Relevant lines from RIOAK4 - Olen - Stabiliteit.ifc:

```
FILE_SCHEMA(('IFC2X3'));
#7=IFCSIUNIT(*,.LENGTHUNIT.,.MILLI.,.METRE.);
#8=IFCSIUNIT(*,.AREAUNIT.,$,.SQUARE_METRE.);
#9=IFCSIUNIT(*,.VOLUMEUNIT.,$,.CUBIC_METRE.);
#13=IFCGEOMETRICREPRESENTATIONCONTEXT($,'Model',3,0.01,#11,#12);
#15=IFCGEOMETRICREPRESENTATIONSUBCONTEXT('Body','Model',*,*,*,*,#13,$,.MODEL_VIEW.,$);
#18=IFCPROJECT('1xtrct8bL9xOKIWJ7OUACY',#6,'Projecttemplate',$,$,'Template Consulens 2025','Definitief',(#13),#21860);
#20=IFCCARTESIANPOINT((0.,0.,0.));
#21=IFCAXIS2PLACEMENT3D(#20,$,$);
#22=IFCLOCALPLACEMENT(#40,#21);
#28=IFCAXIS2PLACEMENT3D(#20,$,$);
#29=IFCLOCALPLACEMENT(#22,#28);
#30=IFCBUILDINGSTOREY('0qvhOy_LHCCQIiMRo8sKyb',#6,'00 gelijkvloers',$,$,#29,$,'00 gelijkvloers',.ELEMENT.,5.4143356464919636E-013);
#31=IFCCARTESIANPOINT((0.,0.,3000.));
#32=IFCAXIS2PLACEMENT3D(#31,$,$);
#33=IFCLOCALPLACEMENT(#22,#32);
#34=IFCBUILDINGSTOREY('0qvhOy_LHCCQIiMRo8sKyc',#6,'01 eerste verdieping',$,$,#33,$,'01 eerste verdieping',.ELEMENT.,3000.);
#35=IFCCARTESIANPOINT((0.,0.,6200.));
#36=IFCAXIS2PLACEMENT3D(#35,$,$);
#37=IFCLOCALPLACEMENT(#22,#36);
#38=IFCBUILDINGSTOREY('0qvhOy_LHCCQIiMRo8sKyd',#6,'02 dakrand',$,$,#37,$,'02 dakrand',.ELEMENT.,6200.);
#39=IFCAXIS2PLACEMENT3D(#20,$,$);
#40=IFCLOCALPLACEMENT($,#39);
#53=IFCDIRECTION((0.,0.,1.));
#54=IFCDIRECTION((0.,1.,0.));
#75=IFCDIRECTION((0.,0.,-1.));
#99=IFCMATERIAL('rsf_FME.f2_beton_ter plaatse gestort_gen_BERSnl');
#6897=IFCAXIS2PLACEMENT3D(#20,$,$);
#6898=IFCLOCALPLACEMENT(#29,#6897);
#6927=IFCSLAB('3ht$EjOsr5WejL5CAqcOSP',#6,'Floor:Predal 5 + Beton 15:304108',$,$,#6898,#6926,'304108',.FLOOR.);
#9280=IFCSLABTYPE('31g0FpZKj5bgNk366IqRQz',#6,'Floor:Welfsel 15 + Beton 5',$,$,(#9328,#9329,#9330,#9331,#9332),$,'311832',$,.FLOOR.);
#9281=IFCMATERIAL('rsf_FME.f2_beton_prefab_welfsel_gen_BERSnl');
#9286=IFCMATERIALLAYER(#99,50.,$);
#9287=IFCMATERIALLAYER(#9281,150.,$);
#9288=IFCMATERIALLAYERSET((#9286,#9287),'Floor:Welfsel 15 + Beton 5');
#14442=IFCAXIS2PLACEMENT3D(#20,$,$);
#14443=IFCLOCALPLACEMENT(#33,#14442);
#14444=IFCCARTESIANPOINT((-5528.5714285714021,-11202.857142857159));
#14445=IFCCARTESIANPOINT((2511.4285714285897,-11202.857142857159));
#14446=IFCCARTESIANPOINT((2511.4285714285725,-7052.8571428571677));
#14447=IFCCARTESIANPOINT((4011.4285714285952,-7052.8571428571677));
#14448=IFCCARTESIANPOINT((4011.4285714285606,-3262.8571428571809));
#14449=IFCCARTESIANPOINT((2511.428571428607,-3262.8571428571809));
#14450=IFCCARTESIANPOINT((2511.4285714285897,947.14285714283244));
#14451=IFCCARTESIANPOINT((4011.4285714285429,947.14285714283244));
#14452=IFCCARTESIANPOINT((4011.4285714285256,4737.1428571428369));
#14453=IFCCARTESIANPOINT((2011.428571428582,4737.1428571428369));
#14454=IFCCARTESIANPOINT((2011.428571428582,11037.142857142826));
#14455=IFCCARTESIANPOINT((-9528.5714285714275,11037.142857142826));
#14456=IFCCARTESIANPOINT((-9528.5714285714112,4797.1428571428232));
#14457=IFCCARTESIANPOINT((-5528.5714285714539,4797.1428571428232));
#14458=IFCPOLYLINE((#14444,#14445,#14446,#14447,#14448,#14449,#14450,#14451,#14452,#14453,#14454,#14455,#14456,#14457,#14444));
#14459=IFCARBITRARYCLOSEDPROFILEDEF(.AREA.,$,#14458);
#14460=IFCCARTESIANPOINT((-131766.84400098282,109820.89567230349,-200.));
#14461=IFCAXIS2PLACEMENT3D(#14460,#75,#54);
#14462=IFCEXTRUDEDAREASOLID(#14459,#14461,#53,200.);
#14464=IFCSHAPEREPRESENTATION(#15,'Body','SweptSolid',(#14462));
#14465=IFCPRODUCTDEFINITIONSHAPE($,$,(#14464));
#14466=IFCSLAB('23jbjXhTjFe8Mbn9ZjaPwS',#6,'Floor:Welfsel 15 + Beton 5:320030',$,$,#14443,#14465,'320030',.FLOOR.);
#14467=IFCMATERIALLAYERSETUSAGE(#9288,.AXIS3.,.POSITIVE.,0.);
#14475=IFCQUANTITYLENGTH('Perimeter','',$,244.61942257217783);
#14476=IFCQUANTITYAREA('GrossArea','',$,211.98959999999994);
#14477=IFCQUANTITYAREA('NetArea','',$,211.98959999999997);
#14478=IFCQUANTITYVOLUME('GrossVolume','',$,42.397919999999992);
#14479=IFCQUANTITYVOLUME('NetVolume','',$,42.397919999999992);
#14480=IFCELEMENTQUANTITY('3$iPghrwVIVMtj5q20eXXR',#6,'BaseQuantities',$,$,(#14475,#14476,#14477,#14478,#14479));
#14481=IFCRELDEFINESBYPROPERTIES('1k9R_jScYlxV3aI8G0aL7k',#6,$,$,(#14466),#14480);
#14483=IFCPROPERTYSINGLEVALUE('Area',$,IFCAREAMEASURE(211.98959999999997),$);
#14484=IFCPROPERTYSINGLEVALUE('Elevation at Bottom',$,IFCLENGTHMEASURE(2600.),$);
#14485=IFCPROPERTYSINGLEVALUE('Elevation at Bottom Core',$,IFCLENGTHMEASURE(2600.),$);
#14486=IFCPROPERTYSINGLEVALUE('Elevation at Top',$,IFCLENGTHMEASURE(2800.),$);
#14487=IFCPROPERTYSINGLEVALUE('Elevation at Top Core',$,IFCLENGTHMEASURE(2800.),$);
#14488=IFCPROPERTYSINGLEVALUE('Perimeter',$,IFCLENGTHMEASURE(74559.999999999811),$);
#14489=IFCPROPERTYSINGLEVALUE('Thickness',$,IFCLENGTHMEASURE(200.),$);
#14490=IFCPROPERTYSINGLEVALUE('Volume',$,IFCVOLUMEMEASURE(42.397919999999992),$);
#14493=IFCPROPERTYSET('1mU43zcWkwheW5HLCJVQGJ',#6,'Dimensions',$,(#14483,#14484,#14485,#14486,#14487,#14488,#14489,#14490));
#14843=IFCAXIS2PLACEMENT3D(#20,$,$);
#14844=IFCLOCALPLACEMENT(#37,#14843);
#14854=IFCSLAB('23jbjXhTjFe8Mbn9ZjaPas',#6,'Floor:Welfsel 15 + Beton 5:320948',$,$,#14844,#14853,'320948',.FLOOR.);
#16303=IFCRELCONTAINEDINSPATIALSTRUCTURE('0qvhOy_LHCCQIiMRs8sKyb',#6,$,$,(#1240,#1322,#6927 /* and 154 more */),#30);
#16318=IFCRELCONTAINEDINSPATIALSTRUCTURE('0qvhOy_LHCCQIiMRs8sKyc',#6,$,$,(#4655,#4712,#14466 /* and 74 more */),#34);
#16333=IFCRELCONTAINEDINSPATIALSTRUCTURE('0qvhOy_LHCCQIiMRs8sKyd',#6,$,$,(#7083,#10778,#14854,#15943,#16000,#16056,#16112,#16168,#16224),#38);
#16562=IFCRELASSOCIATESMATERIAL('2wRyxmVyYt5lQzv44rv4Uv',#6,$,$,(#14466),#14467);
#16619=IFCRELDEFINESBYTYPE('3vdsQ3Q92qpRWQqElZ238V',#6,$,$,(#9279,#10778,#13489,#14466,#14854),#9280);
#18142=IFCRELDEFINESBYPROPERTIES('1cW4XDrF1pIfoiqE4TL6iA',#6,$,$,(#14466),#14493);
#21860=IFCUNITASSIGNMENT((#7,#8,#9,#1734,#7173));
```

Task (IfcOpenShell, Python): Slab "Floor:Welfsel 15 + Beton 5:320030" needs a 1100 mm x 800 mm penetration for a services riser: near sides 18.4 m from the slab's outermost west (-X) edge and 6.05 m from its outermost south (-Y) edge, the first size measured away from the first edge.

```python
import numpy as np
import ifcopenshell
import ifcopenshell.api.feature
import ifcopenshell.api.geometry
import ifcopenshell.api.pset
import ifcopenshell.api.root
import ifcopenshell.geom
import ifcopenshell.util.element
import ifcopenshell.util.placement
import ifcopenshell.util.representation
import ifcopenshell.util.shape
import ifcopenshell.util.unit

model = ifcopenshell.open("RIOAK4 - Olen - Stabiliteit.ifc")
unit_scale = ifcopenshell.util.unit.calculate_unit_scale(model)
area_scale = ifcopenshell.util.unit.calculate_unit_scale(model, "AREAUNIT")
volume_scale = ifcopenshell.util.unit.calculate_unit_scale(model, "VOLUMEUNIT")
settings = ifcopenshell.geom.settings()


def volume(element):
    """Net volume in cubic metres, openings subtracted."""
    shape = ifcopenshell.geom.create_shape(settings, element)
    return ifcopenshell.util.shape.get_volume(shape.geometry)


slab = model.by_guid("23jbjXhTjFe8Mbn9ZjaPwS")
before = volume(slab)

# Extent in the slab's own axes, in metres. The edges named are its -X and -Y sides.
slab_shape = ifcopenshell.geom.create_shape(settings, slab)
vertices = ifcopenshell.util.shape.get_vertices(slab_shape.geometry)
x_min, y_min, bottom = vertices.min(axis=0)
top = vertices[:, 2].max()

opening = ifcopenshell.api.root.create_entity(model, ifc_class="IfcOpeningElement", name="Services riser opening")
context = ifcopenshell.util.representation.get_context(model, "Model", "Body", "MODEL_VIEW")
width, depth = 1.1, 0.8
outline = [(0.0, 0.0), (width, 0.0), (width, depth), (0.0, depth), (0.0, 0.0)]
# Overshoot both faces by 50 mm so the cut is clean.
shape = ifcopenshell.api.geometry.add_slab_representation(
    model, context=context, depth=top - bottom + 0.1, polyline=outline
)
ifcopenshell.api.geometry.assign_representation(model, product=opening, representation=shape)

matrix = ifcopenshell.util.placement.get_local_placement(slab.ObjectPlacement)
matrix[:, 3] = matrix @ np.append(np.array([x_min + 18.4, y_min + 6.05, bottom - 0.05]) / unit_scale, 1.0)
ifcopenshell.api.geometry.edit_object_placement(model, product=opening, matrix=matrix, is_si=False)
ifcopenshell.api.feature.add_feature(model, feature=opening, element=slab)

after = volume(slab)

# Update the slab's stored quantities.
qto = model.by_id(ifcopenshell.util.element.get_pset(slab, "BaseQuantities", should_inherit=False)["id"])
ifcopenshell.api.pset.edit_qto(model, qto=qto, properties={
    "NetArea": after / (top - bottom) / area_scale,
    "NetVolume": after / volume_scale,
})
pset = model.by_id(ifcopenshell.util.element.get_pset(slab, "Dimensions", should_inherit=False)["id"])
ifcopenshell.api.pset.edit_pset(model, pset=pset, properties={
    "Area": model.create_entity("IfcAreaMeasure", after / (top - bottom) / area_scale),
    "Volume": model.create_entity("IfcVolumeMeasure", after / volume_scale),
})

print(f"slab volume {before:.3f} -> {after:.3f} m3")

model.write("RIOAK4 - Olen - Stabiliteit_updated.ifc")
```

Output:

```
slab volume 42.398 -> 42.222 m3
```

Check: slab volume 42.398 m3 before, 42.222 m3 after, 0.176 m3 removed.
